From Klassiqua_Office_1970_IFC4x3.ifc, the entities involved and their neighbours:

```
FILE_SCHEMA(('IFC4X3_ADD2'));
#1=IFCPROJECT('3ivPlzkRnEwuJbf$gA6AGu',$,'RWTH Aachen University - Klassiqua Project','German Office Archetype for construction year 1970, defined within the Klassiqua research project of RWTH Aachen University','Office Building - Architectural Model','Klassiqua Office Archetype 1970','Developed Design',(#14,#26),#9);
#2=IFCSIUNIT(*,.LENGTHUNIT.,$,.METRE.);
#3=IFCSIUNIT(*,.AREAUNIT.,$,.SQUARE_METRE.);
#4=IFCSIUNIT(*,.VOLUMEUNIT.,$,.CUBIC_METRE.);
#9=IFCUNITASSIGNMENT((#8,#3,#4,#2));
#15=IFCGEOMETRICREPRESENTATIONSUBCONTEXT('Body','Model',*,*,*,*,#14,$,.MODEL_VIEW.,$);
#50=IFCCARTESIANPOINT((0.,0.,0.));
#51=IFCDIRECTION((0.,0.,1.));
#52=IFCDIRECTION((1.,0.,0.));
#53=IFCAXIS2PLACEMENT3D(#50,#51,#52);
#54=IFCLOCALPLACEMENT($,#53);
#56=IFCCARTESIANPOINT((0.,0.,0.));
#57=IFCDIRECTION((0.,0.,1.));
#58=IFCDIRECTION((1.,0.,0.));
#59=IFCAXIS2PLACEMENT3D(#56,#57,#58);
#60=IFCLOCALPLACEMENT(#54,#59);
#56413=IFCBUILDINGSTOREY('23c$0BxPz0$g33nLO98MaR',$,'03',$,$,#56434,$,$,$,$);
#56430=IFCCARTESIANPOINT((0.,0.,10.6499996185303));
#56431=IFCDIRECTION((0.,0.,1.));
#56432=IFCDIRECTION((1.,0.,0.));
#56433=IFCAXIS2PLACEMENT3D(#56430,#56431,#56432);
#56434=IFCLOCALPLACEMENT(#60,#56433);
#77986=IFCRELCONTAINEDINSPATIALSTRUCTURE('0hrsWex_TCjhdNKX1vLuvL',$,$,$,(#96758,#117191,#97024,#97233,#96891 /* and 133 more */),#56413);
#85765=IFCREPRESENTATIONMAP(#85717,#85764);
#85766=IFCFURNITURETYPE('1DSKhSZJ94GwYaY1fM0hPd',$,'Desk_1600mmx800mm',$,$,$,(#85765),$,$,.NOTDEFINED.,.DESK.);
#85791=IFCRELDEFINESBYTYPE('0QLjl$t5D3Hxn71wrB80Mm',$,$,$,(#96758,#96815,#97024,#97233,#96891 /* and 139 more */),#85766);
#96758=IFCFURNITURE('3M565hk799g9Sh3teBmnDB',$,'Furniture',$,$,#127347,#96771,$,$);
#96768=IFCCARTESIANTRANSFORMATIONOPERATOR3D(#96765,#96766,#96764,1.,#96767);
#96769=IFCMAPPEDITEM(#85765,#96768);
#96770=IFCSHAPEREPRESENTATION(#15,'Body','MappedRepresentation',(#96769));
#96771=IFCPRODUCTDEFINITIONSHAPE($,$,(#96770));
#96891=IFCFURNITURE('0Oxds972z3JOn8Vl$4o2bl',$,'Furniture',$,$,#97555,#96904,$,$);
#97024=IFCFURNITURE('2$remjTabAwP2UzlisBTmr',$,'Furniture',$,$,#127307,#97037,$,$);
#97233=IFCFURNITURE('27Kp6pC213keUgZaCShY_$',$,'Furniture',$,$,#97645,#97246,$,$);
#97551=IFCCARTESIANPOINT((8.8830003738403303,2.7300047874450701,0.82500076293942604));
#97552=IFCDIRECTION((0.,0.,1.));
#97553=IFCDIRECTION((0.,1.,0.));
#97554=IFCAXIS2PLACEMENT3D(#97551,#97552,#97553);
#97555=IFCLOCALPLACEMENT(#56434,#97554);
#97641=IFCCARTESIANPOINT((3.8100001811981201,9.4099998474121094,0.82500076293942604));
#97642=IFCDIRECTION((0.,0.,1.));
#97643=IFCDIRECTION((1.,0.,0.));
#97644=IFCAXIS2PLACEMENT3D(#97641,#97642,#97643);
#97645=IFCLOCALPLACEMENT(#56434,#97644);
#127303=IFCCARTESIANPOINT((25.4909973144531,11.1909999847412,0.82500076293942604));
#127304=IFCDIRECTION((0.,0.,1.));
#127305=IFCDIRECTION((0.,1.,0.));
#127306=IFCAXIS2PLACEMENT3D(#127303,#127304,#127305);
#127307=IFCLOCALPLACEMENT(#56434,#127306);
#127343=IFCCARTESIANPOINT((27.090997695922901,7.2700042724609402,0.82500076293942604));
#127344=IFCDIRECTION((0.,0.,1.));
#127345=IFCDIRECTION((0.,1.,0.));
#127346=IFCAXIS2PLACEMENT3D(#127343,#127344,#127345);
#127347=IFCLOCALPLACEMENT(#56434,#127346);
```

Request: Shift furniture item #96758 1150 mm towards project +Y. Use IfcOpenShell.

```python
import ifcopenshell
import ifcopenshell.api.geometry
import ifcopenshell.util.placement
import ifcopenshell.util.unit

model = ifcopenshell.open("Klassiqua_Office_1970_IFC4x3.ifc")
unit_scale = ifcopenshell.util.unit.calculate_unit_scale(model)

item = model.by_guid("3M565hk799g9Sh3teBmnDB")
matrix = ifcopenshell.util.placement.get_local_placement(item.ObjectPlacement)
matrix[1, 3] += 1.15 / unit_scale
ifcopenshell.api.geometry.edit_object_placement(model, product=item, matrix=matrix, is_si=False)

print(ifcopenshell.util.placement.get_local_placement(item.ObjectPlacement).round(3) + 0.0)

model.write("Klassiqua_Office_1970_IFC4x3_v2.ifc")
```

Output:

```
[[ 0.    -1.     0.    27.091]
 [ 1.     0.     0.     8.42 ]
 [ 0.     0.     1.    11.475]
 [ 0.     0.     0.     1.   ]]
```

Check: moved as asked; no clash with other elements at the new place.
